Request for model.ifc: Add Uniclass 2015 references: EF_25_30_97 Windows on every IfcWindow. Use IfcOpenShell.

First a look at what the model holds.

```python
import ifcopenshell

model = ifcopenshell.open("model.ifc")
print(model.schema)
print("classifications:", [c.Name for c in model.by_type("IfcClassification")])
for ifc_class in ("IfcDoor", "IfcRoof", "IfcStair", "IfcWall", "IfcWindow"):
    print(ifc_class, len(model.by_type(ifc_class)))
```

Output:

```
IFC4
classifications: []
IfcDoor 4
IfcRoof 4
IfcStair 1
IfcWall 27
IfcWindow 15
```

```python
import ifcopenshell
import ifcopenshell.api.classification

model = ifcopenshell.open("model.ifc")

system = ifcopenshell.api.classification.add_classification(model, classification="Uniclass 2015")

codes = {
    "IfcWindow": ("EF_25_30_97", "Windows"),
}
for ifc_class, (code, name) in codes.items():
    products = model.by_type(ifc_class)
    ifcopenshell.api.classification.add_reference(
        model, products=products, classification=system, identification=code, name=name
    )
    print(code, len(products))

model.write("model_edited.ifc")
```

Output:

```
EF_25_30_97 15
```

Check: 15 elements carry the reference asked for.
